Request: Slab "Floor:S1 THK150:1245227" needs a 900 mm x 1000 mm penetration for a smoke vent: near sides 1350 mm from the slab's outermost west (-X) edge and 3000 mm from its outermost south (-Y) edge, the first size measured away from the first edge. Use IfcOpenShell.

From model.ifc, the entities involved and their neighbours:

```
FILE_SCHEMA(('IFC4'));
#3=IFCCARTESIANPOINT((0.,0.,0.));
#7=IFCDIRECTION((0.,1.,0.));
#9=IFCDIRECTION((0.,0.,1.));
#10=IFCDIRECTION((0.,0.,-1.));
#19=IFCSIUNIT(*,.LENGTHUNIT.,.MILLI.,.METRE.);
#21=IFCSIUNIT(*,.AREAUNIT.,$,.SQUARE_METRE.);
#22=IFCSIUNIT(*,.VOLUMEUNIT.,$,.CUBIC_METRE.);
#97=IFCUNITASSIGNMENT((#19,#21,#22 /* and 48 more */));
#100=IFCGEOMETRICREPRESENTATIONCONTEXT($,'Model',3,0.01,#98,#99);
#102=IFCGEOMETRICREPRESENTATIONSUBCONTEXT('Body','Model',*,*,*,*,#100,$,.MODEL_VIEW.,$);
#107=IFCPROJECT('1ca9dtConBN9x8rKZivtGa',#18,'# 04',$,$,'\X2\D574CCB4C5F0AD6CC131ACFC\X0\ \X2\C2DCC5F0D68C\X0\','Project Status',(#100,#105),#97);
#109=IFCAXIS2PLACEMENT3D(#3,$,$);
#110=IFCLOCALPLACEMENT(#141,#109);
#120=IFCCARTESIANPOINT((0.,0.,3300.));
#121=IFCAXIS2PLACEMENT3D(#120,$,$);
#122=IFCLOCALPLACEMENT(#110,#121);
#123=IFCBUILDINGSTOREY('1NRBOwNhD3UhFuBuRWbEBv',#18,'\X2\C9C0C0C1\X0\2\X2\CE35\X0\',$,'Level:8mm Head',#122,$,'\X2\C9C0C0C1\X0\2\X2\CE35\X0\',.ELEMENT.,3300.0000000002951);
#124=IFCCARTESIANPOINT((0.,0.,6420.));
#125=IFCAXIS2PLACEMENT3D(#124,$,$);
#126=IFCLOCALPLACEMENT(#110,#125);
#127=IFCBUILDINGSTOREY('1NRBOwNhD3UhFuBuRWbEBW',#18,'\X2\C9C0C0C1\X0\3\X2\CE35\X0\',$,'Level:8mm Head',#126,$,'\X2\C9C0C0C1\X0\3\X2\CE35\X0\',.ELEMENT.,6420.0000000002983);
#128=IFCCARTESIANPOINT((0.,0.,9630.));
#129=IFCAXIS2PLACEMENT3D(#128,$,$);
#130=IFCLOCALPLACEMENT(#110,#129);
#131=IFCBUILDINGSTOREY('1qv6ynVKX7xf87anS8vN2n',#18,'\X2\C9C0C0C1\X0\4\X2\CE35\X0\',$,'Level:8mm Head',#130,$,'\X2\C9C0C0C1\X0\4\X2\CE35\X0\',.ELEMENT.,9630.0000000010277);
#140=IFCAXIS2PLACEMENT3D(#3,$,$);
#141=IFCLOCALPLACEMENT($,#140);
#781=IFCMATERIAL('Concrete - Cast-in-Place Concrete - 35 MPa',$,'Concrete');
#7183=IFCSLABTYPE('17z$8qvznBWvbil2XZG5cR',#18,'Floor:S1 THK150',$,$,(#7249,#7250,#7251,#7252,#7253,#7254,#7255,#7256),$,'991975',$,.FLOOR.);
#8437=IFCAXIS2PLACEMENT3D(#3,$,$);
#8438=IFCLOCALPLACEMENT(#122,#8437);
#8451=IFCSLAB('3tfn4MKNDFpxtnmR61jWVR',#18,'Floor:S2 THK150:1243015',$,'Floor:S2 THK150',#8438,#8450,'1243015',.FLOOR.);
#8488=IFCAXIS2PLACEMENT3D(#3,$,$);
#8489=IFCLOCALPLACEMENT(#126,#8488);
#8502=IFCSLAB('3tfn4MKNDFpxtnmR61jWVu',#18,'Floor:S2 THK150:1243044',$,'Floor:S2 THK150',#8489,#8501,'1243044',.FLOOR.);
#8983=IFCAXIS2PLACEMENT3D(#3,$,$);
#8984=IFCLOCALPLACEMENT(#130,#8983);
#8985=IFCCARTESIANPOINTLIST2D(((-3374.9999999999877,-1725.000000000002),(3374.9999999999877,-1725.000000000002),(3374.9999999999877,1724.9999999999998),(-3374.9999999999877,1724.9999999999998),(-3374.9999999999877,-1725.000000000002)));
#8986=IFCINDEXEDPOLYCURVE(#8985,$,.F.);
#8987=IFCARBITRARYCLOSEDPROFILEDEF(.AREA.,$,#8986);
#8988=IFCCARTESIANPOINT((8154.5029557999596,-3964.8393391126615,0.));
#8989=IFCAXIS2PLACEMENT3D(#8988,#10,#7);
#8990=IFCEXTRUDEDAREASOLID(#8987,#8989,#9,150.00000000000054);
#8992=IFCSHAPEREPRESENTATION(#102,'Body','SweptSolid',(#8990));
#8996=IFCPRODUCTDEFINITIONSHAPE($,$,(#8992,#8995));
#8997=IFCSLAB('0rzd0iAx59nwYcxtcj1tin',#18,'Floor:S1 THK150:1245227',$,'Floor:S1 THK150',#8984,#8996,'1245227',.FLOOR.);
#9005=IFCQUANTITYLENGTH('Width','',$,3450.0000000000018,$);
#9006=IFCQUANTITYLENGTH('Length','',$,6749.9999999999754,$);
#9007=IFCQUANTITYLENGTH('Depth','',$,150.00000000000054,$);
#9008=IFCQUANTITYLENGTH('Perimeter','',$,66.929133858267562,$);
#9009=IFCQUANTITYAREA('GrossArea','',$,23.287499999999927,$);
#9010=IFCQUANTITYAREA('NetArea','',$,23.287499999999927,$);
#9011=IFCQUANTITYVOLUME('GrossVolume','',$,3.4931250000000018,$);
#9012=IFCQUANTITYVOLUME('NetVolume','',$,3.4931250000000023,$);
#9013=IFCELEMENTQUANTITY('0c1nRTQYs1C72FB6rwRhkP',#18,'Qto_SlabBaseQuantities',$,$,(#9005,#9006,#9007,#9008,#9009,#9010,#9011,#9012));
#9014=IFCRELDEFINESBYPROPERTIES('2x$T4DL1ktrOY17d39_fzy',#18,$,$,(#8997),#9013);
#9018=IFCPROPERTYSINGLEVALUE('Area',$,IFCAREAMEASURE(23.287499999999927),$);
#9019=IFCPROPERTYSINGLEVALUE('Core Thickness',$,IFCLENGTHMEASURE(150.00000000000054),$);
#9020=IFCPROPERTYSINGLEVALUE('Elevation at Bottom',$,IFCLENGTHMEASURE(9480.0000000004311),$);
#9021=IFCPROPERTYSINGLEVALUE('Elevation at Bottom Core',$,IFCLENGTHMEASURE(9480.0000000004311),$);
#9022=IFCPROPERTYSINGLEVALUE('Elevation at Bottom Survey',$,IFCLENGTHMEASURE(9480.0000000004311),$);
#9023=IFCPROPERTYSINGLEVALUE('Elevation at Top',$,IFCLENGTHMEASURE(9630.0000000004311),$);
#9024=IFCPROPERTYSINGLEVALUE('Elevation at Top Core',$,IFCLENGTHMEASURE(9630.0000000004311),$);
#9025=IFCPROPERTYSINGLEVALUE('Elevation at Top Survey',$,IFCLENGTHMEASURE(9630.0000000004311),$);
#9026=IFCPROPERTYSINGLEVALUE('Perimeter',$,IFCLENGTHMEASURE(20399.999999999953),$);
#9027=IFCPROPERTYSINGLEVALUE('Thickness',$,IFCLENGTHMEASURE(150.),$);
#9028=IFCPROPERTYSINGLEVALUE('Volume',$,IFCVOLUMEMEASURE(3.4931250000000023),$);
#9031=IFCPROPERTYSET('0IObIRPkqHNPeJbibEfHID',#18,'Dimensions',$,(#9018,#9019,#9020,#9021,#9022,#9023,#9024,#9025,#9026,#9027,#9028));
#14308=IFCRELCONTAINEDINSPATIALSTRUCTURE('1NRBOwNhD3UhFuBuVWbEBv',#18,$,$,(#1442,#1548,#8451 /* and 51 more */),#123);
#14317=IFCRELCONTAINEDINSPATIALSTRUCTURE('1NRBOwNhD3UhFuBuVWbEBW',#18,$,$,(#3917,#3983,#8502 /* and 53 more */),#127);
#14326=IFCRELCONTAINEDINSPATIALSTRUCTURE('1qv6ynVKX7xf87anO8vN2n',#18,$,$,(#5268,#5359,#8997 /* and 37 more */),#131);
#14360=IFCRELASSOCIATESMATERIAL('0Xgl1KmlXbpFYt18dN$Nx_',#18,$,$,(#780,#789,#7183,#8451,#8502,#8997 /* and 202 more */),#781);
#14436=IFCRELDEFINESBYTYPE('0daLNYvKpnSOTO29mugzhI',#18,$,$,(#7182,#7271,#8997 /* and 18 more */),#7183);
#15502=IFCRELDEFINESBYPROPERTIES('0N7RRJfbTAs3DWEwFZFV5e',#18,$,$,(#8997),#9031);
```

```python
import numpy as np
import ifcopenshell
import ifcopenshell.api.feature
import ifcopenshell.api.geometry
import ifcopenshell.api.pset
import ifcopenshell.api.root
import ifcopenshell.geom
import ifcopenshell.util.element
import ifcopenshell.util.placement
import ifcopenshell.util.representation
import ifcopenshell.util.shape
import ifcopenshell.util.unit

model = ifcopenshell.open("model.ifc")
unit_scale = ifcopenshell.util.unit.calculate_unit_scale(model)
area_scale = ifcopenshell.util.unit.calculate_unit_scale(model, "AREAUNIT")
volume_scale = ifcopenshell.util.unit.calculate_unit_scale(model, "VOLUMEUNIT")
settings = ifcopenshell.geom.settings()


def volume(element):
    """Net volume in cubic metres, openings subtracted."""
    shape = ifcopenshell.geom.create_shape(settings, element)
    return ifcopenshell.util.shape.get_volume(shape.geometry)


slab = model.by_guid("0rzd0iAx59nwYcxtcj1tin")
before = volume(slab)

# Extent in the slab's own axes, in metres. The edges named are its -X and -Y sides.
slab_shape = ifcopenshell.geom.create_shape(settings, slab)
vertices = ifcopenshell.util.shape.get_vertices(slab_shape.geometry)
x_min, y_min, bottom = vertices.min(axis=0)
top = vertices[:, 2].max()

opening = ifcopenshell.api.root.create_entity(model, ifc_class="IfcOpeningElement", name="Smoke vent opening", predefined_type="OPENING")
context = ifcopenshell.util.representation.get_context(model, "Model", "Body", "MODEL_VIEW")
width, depth = 0.9, 1
outline = [(0.0, 0.0), (width, 0.0), (width, depth), (0.0, depth), (0.0, 0.0)]
# Overshoot both faces by 50 mm so the cut is clean.
shape = ifcopenshell.api.geometry.add_slab_representation(
    model, context=context, depth=top - bottom + 0.1, polyline=outline
)
ifcopenshell.api.geometry.assign_representation(model, product=opening, representation=shape)

matrix = ifcopenshell.util.placement.get_local_placement(slab.ObjectPlacement)
matrix[:, 3] = matrix @ np.append(np.array([x_min + 1.35, y_min + 3, bottom - 0.05]) / unit_scale, 1.0)
ifcopenshell.api.geometry.edit_object_placement(model, product=opening, matrix=matrix, is_si=False)
ifcopenshell.api.feature.add_feature(model, feature=opening, element=slab)

after = volume(slab)

# Update the slab's stored quantities.
qto = model.by_id(ifcopenshell.util.element.get_pset(slab, "Qto_SlabBaseQuantities", should_inherit=False)["id"])
ifcopenshell.api.pset.edit_qto(model, qto=qto, properties={
    "NetArea": after / (top - bottom) / area_scale,
    "NetVolume": after / volume_scale,
})
pset = model.by_id(ifcopenshell.util.element.get_pset(slab, "Dimensions", should_inherit=False)["id"])
ifcopenshell.api.pset.edit_pset(model, pset=pset, properties={
    "Area": model.create_entity("IfcAreaMeasure", after / (top - bottom) / area_scale),
    "Volume": model.create_entity("IfcVolumeMeasure", after / volume_scale),
})

print(f"slab volume {before:.3f} -> {after:.3f} m3")

model.write("model-out.ifc")
```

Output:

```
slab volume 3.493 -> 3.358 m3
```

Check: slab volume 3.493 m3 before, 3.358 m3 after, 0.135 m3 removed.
